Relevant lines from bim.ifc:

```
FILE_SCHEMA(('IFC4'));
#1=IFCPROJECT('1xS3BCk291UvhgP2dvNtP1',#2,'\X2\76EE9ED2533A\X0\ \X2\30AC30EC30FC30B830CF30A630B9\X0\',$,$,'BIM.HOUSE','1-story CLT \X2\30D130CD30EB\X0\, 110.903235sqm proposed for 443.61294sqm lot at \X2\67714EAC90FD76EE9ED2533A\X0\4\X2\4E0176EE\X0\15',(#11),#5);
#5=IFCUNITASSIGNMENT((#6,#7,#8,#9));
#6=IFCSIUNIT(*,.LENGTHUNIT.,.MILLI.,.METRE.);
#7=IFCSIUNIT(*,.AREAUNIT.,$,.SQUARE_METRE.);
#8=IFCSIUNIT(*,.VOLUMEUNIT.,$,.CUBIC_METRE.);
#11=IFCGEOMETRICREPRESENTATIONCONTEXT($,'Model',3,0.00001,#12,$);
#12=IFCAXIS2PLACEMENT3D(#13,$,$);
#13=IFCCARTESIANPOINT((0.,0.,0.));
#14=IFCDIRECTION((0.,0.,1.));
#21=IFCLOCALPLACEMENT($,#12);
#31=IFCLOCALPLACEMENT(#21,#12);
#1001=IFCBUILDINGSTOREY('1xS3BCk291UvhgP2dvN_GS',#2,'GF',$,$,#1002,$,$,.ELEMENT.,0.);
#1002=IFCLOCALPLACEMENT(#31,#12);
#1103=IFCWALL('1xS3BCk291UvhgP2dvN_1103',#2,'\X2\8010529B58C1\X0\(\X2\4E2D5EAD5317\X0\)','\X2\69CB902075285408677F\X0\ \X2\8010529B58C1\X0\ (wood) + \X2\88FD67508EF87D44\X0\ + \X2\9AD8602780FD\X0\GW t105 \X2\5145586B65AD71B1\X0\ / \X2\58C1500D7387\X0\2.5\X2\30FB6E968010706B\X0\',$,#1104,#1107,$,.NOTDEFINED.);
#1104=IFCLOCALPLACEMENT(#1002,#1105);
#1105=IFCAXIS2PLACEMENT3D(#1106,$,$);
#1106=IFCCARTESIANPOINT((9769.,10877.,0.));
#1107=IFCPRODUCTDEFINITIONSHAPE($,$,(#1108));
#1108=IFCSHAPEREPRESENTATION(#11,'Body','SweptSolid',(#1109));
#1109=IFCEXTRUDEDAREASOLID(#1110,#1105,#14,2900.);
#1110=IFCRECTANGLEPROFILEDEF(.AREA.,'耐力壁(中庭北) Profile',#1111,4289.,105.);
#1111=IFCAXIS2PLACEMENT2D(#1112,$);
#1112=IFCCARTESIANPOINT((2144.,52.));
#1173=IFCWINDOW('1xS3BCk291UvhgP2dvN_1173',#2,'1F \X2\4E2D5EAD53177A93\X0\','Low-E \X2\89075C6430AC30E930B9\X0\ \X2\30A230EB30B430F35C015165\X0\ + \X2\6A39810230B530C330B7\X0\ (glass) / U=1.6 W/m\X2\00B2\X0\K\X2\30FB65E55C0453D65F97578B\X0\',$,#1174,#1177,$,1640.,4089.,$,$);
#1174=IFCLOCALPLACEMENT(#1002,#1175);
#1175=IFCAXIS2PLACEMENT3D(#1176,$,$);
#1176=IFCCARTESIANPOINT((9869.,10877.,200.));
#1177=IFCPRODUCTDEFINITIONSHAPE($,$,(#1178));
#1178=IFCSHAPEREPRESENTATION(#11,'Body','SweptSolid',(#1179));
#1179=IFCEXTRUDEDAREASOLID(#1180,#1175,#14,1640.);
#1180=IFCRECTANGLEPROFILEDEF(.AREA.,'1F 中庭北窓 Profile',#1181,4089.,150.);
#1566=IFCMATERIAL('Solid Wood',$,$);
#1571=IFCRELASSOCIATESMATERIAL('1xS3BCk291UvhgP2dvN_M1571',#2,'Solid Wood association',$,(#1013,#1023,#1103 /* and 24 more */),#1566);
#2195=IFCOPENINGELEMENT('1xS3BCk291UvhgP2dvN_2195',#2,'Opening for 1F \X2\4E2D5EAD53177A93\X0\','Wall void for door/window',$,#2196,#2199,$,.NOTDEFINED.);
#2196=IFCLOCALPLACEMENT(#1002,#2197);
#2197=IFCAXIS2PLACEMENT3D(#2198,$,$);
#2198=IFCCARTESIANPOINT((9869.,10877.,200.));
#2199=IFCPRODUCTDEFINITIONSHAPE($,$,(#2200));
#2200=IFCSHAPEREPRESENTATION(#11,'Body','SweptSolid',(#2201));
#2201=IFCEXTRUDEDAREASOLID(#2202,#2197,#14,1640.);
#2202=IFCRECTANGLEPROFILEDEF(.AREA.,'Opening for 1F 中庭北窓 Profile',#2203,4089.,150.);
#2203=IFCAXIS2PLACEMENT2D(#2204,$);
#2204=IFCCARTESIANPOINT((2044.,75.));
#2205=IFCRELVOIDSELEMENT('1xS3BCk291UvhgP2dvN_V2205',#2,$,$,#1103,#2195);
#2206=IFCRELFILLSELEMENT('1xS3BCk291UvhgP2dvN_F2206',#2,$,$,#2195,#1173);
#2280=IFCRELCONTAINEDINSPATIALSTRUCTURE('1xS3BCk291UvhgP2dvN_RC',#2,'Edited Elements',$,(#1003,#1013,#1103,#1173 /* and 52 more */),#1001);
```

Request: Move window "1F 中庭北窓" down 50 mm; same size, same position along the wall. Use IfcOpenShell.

```python
import numpy as np
import ifcopenshell
import ifcopenshell.api.geometry
import ifcopenshell.util.placement
import ifcopenshell.util.unit

model = ifcopenshell.open("bim.ifc")
unit_scale = ifcopenshell.util.unit.calculate_unit_scale(model)

window = model.by_guid("1xS3BCk291UvhgP2dvN_1173")
opening = window.FillsVoids[0].RelatingOpeningElement
dz = -50.0

shift = np.array([0.0, 0.0, dz])
# The window is not placed relative to its opening, so move both.
for product in (opening, window):
    matrix = ifcopenshell.util.placement.get_local_placement(product.ObjectPlacement)
    matrix[:3, 3] += shift
    ifcopenshell.api.geometry.edit_object_placement(model, product=product, matrix=matrix, is_si=False)

print(f"moved by {dz * unit_scale:+.3f} m")

model.write("bim_edited.ifc")
```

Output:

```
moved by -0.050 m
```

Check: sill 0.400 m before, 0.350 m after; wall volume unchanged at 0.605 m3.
